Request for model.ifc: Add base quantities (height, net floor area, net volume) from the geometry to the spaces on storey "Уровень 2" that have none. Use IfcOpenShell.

First a look at what the model holds.

```python
import ifcopenshell
import ifcopenshell.util.element
import ifcopenshell.util.unit

model = ifcopenshell.open("model.ifc")
print(model.schema)
for unit_type in ("LENGTHUNIT", "AREAUNIT", "VOLUMEUNIT"):
    print(unit_type, ifcopenshell.util.unit.calculate_unit_scale(model, unit_type))
storey = next(s for s in model.by_type("IfcBuildingStorey") if s.Name == "Уровень 2")
spaces = [e for e in ifcopenshell.util.element.get_decomposition(storey) if e.is_a("IfcSpace")]
for e in sorted(spaces, key=lambda e: e.id()):
    print(e.id(), e.is_a(), e.Name, list(ifcopenshell.util.element.get_psets(e, qtos_only=True)), sep=" | ")
```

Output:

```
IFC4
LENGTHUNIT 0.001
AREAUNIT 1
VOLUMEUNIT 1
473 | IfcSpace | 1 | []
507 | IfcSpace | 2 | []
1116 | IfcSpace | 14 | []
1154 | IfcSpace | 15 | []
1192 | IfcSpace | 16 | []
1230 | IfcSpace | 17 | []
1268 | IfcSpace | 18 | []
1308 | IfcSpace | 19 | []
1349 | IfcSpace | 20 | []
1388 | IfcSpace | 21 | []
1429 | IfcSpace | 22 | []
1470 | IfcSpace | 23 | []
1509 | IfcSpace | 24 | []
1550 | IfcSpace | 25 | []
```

```python
import ifcopenshell
import ifcopenshell.api.pset
import ifcopenshell.geom
import ifcopenshell.util.element
import ifcopenshell.util.shape
import ifcopenshell.util.unit

model = ifcopenshell.open("model.ifc")
unit_scale = ifcopenshell.util.unit.calculate_unit_scale(model)
area_scale = ifcopenshell.util.unit.calculate_unit_scale(model, "AREAUNIT")
volume_scale = ifcopenshell.util.unit.calculate_unit_scale(model, "VOLUMEUNIT")
settings = ifcopenshell.geom.settings()

storey = next(s for s in model.by_type("IfcBuildingStorey") if s.Name == "Уровень 2")
spaces = [e for e in ifcopenshell.util.element.get_decomposition(storey) if e.is_a("IfcSpace")]

for e in sorted(spaces, key=lambda e: e.id()):
    if ifcopenshell.util.element.get_psets(e, qtos_only=True, should_inherit=False):
        continue
    # Geometry comes back in metres, in the element's own axes.
    shape = ifcopenshell.geom.create_shape(settings, e)
    values = {
        "Height": ifcopenshell.util.shape.get_z(shape.geometry) / unit_scale,
        "NetFloorArea": ifcopenshell.util.shape.get_footprint_area(shape.geometry) / area_scale,
        "NetVolume": ifcopenshell.util.shape.get_volume(shape.geometry) / volume_scale,
    }
    qto = ifcopenshell.api.pset.add_qto(model, product=e, name="Qto_SpaceBaseQuantities")
    ifcopenshell.api.pset.edit_qto(model, qto=qto, properties=values)
    print(e.id(), {k: round(v, 3) for k, v in values.items()})

model.write("model_v2.ifc")
```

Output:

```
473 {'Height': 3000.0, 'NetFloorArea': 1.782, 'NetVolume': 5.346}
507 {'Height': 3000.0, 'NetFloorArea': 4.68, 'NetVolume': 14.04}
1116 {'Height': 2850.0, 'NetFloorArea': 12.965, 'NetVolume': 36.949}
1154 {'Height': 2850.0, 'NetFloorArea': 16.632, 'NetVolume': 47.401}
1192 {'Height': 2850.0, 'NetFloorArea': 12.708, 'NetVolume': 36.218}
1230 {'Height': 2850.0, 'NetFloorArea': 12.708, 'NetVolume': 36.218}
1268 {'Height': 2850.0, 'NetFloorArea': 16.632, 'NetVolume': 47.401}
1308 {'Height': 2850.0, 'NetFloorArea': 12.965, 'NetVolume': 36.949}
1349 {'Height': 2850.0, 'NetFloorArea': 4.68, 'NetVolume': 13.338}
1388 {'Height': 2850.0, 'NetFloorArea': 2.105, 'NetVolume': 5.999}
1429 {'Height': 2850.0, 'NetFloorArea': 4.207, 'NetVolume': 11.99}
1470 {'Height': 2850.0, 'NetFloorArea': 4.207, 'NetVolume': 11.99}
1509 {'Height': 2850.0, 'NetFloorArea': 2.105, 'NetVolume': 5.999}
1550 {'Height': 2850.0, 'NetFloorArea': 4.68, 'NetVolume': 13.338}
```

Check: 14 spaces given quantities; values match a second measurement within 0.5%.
